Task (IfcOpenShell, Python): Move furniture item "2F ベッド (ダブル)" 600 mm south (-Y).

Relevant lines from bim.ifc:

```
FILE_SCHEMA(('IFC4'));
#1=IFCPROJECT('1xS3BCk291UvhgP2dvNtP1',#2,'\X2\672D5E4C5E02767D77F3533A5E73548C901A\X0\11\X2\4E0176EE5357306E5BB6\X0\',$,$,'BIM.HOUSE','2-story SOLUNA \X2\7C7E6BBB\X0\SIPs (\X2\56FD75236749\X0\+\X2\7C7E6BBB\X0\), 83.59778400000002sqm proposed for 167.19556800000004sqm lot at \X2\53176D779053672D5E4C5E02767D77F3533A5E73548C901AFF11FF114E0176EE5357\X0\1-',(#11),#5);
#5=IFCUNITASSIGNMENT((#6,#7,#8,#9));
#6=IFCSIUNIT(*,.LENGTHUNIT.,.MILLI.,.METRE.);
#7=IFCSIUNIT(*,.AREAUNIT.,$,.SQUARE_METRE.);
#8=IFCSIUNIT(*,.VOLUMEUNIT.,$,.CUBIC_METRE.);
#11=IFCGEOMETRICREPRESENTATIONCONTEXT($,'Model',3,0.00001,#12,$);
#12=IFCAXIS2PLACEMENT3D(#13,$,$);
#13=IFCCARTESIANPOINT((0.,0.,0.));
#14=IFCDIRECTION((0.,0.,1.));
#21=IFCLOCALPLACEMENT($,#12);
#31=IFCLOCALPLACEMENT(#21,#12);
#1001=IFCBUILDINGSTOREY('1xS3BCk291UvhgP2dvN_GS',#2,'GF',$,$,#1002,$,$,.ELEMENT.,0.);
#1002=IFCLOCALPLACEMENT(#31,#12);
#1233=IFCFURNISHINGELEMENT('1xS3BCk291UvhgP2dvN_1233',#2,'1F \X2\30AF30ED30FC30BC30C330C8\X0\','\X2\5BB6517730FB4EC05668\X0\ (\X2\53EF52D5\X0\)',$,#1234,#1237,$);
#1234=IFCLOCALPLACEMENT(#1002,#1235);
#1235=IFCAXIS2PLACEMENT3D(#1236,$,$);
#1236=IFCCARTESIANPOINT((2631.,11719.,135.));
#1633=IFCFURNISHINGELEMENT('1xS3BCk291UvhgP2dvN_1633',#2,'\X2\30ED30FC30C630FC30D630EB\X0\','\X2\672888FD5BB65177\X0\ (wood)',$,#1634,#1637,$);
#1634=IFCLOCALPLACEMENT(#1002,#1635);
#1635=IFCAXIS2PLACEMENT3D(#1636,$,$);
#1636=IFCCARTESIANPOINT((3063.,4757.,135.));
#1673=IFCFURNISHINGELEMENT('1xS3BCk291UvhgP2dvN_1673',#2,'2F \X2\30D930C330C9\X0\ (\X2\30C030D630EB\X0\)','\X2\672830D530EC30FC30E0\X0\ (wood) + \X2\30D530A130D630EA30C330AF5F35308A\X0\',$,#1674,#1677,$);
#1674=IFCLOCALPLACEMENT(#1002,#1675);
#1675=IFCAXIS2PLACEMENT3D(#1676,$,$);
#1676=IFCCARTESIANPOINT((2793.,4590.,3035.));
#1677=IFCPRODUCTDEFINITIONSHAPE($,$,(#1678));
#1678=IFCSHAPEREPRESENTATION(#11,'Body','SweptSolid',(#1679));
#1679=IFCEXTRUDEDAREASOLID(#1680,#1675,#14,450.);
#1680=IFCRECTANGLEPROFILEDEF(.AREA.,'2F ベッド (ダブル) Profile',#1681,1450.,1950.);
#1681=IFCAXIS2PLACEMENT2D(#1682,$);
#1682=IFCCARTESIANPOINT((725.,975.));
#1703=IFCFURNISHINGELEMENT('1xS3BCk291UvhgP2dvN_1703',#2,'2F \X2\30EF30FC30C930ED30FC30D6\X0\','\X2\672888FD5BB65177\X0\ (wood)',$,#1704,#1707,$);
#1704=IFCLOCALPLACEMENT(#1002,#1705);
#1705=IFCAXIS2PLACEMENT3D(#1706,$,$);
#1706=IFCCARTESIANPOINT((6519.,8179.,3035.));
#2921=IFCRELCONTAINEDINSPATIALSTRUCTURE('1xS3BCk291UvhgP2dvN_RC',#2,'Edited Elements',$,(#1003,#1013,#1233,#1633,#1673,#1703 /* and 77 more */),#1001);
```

```python
import ifcopenshell
import ifcopenshell.api.geometry
import ifcopenshell.util.placement
import ifcopenshell.util.unit

model = ifcopenshell.open("bim.ifc")
unit_scale = ifcopenshell.util.unit.calculate_unit_scale(model)

item = model.by_guid("1xS3BCk291UvhgP2dvN_1673")
matrix = ifcopenshell.util.placement.get_local_placement(item.ObjectPlacement)
matrix[1, 3] -= 0.6 / unit_scale
ifcopenshell.api.geometry.edit_object_placement(model, product=item, matrix=matrix, is_si=False)

print(ifcopenshell.util.placement.get_local_placement(item.ObjectPlacement).round(3) + 0.0)

model.write("bim_updated.ifc")
```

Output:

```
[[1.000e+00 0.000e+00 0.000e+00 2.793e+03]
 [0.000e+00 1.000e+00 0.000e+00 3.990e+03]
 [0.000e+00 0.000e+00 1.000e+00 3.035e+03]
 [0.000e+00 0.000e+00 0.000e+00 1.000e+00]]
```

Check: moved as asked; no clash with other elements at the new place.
